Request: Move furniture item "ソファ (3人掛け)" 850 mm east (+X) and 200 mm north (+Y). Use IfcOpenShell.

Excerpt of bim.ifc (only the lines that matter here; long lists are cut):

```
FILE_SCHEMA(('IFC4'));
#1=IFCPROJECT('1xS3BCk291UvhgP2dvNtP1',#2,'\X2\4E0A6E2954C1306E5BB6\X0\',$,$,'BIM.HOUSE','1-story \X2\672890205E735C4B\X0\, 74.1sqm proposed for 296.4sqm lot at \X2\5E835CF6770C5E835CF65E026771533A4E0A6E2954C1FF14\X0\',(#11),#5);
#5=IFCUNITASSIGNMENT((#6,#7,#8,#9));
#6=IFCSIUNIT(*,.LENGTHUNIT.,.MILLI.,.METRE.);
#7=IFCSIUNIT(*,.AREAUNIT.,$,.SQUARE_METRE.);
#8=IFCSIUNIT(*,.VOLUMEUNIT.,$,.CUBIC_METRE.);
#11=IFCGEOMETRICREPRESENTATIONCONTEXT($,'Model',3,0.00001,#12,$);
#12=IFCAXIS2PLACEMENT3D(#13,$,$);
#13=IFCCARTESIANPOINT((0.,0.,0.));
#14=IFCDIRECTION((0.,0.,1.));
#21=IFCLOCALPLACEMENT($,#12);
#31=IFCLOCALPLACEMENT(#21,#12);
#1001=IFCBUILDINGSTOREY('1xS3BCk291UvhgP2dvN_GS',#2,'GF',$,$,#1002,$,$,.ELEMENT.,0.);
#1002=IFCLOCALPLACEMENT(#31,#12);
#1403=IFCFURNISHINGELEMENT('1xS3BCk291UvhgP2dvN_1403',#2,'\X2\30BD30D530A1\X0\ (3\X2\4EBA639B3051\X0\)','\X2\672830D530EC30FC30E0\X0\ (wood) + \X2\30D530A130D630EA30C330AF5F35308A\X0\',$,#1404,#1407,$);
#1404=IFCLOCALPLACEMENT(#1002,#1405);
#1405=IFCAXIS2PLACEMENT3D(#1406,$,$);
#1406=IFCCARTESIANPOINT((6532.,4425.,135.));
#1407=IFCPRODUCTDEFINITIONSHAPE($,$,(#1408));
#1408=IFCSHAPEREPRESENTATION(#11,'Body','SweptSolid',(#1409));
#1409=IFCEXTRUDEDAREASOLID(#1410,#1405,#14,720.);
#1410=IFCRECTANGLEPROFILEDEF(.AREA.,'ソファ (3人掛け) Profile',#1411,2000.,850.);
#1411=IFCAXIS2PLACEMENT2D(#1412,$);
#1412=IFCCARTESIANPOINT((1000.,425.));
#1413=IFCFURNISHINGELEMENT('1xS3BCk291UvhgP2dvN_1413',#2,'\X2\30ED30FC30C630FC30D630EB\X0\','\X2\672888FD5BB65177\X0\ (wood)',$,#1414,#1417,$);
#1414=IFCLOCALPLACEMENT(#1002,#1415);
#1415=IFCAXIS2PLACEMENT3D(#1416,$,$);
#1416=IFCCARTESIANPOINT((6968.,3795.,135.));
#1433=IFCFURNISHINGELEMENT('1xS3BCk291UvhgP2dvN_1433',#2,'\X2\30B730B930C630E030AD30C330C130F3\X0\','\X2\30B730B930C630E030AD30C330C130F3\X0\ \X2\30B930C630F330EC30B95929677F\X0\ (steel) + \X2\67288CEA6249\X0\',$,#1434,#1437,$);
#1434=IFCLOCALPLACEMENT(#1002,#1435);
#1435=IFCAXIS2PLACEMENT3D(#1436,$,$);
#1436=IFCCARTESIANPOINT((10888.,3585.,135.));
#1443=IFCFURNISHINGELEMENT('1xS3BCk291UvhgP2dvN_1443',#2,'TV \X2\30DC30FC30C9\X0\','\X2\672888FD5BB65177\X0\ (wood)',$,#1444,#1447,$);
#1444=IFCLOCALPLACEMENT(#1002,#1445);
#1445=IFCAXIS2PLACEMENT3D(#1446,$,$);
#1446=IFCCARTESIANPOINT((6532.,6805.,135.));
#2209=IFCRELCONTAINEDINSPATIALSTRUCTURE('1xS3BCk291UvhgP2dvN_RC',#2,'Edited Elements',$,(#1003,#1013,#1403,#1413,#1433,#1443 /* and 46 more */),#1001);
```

```python
import ifcopenshell
import ifcopenshell.api.geometry
import ifcopenshell.util.placement

model = ifcopenshell.open("bim.ifc")

item = model.by_guid("1xS3BCk291UvhgP2dvN_1403")
matrix = ifcopenshell.util.placement.get_local_placement(item.ObjectPlacement)
matrix[0, 3] += 850.0
matrix[1, 3] += 200.0
ifcopenshell.api.geometry.edit_object_placement(model, product=item, matrix=matrix, is_si=False)

print(ifcopenshell.util.placement.get_local_placement(item.ObjectPlacement).round(3) + 0.0)

model.write("bim_updated.ifc")
```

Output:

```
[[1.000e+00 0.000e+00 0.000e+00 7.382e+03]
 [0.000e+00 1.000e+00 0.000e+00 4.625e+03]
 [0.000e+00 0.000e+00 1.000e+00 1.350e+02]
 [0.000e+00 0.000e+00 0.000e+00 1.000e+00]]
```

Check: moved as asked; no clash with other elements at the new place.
